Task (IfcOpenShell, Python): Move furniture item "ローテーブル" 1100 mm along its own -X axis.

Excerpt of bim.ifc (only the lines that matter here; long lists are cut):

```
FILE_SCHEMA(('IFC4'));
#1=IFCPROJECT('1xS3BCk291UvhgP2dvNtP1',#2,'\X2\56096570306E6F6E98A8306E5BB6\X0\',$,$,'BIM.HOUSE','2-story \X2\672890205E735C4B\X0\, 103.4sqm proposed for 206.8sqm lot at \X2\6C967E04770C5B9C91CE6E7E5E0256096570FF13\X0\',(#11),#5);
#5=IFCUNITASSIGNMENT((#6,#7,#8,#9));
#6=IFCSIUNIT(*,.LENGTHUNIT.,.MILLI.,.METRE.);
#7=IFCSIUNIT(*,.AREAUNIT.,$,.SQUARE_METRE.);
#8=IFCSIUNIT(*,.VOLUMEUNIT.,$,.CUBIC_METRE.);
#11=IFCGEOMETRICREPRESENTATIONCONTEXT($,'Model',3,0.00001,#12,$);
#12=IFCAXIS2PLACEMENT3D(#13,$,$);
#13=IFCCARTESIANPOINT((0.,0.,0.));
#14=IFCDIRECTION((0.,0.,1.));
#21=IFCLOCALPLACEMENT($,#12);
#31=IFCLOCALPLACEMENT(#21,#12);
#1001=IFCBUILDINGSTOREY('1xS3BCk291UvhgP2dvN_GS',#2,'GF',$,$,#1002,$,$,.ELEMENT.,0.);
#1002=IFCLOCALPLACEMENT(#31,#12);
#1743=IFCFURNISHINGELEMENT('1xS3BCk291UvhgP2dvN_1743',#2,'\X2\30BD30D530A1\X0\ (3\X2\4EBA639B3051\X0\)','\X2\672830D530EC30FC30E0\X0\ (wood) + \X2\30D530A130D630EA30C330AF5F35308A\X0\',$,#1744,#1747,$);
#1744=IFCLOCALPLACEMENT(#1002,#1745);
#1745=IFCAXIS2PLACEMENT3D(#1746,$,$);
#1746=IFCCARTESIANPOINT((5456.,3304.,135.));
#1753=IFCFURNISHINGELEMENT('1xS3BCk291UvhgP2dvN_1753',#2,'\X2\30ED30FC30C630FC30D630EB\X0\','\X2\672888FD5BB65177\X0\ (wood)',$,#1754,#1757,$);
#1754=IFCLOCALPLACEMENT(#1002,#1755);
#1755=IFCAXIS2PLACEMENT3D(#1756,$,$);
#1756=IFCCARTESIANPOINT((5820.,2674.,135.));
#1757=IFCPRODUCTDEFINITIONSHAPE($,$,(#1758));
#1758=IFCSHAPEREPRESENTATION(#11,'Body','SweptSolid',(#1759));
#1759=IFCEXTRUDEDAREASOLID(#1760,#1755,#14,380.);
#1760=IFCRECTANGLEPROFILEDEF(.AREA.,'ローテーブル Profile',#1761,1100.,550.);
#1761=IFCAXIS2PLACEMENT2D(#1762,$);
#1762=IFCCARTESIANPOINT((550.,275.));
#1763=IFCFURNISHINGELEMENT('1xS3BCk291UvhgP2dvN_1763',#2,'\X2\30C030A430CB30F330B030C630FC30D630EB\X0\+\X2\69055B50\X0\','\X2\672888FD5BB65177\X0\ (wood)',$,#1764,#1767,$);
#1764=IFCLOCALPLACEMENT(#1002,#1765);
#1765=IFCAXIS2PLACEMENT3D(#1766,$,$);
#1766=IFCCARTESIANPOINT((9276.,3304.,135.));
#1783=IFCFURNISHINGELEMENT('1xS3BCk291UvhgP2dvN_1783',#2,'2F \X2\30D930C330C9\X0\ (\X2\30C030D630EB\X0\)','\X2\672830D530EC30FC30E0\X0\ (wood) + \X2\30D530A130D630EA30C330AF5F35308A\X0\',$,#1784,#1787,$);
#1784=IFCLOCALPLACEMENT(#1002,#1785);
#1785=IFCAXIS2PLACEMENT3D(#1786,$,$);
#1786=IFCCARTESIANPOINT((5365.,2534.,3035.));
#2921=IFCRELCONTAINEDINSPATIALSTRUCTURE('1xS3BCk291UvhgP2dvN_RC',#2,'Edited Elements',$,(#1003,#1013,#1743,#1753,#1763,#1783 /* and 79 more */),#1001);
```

```python
import ifcopenshell
import ifcopenshell.api.geometry
import ifcopenshell.util.placement
import ifcopenshell.util.unit

model = ifcopenshell.open("bim.ifc")
unit_scale = ifcopenshell.util.unit.calculate_unit_scale(model)

item = model.by_guid("1xS3BCk291UvhgP2dvN_1753")
matrix = ifcopenshell.util.placement.get_local_placement(item.ObjectPlacement)
matrix[:3, 3] -= matrix[:3, 0] * 1.1 / unit_scale
ifcopenshell.api.geometry.edit_object_placement(model, product=item, matrix=matrix, is_si=False)

print(ifcopenshell.util.placement.get_local_placement(item.ObjectPlacement).round(3) + 0.0)

model.write("bim_edited.ifc")
```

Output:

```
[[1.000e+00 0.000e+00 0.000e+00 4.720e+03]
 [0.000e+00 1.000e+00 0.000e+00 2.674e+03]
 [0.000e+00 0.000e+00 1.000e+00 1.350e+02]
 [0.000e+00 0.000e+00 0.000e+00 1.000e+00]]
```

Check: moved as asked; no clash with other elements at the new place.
